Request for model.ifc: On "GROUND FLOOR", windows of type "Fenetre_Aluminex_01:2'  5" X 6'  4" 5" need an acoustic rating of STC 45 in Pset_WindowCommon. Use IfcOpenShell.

First a look at what the model holds.

```python
import ifcopenshell
import ifcopenshell.util.element

model = ifcopenshell.open("model.ifc")
print(model.schema)
storey = next(s for s in model.by_type("IfcBuildingStorey") if s.Name == "GROUND FLOOR")
windows = [e for e in ifcopenshell.util.element.get_decomposition(storey) if e.is_a("IfcWindow")]
seen = {}
for e in windows:
    element_type = ifcopenshell.util.element.get_type(e)
    key = (element_type.Name if element_type != e and element_type else None, ifcopenshell.util.element.get_pset(e, "Pset_WindowCommon", "AcousticRating"))
    seen[key] = seen.get(key, 0) + 1
for (name, value), count in sorted(seen.items(), key=str):
    print(count, "x", name, "|", value)
```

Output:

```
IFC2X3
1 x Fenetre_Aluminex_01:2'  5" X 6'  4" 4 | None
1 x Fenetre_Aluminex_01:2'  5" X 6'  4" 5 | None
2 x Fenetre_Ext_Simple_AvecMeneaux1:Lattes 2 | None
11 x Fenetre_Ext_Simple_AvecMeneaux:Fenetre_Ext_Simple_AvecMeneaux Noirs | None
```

```python
import ifcopenshell
import ifcopenshell.api.pset
import ifcopenshell.util.element

model = ifcopenshell.open("model.ifc")

storey = next(s for s in model.by_type("IfcBuildingStorey") if s.Name == "GROUND FLOOR")
windows = [e for e in ifcopenshell.util.element.get_decomposition(storey) if e.is_a("IfcWindow")]

count = 0
for e in windows:
    element_type = ifcopenshell.util.element.get_type(e)
    if element_type in (None, e) or element_type.Name != 'Fenetre_Aluminex_01:2\'  5" X 6\'  4" 5':
        continue
    # add_pset returns the element's existing set when there is one.
    pset = ifcopenshell.api.pset.add_pset(model, product=e, name="Pset_WindowCommon")
    ifcopenshell.api.pset.edit_pset(model, pset=pset, properties={"AcousticRating": "STC 45"})
    count += 1

print(count, "windows updated")

model.write("model_edited.ifc")
```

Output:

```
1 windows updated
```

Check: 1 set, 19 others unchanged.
